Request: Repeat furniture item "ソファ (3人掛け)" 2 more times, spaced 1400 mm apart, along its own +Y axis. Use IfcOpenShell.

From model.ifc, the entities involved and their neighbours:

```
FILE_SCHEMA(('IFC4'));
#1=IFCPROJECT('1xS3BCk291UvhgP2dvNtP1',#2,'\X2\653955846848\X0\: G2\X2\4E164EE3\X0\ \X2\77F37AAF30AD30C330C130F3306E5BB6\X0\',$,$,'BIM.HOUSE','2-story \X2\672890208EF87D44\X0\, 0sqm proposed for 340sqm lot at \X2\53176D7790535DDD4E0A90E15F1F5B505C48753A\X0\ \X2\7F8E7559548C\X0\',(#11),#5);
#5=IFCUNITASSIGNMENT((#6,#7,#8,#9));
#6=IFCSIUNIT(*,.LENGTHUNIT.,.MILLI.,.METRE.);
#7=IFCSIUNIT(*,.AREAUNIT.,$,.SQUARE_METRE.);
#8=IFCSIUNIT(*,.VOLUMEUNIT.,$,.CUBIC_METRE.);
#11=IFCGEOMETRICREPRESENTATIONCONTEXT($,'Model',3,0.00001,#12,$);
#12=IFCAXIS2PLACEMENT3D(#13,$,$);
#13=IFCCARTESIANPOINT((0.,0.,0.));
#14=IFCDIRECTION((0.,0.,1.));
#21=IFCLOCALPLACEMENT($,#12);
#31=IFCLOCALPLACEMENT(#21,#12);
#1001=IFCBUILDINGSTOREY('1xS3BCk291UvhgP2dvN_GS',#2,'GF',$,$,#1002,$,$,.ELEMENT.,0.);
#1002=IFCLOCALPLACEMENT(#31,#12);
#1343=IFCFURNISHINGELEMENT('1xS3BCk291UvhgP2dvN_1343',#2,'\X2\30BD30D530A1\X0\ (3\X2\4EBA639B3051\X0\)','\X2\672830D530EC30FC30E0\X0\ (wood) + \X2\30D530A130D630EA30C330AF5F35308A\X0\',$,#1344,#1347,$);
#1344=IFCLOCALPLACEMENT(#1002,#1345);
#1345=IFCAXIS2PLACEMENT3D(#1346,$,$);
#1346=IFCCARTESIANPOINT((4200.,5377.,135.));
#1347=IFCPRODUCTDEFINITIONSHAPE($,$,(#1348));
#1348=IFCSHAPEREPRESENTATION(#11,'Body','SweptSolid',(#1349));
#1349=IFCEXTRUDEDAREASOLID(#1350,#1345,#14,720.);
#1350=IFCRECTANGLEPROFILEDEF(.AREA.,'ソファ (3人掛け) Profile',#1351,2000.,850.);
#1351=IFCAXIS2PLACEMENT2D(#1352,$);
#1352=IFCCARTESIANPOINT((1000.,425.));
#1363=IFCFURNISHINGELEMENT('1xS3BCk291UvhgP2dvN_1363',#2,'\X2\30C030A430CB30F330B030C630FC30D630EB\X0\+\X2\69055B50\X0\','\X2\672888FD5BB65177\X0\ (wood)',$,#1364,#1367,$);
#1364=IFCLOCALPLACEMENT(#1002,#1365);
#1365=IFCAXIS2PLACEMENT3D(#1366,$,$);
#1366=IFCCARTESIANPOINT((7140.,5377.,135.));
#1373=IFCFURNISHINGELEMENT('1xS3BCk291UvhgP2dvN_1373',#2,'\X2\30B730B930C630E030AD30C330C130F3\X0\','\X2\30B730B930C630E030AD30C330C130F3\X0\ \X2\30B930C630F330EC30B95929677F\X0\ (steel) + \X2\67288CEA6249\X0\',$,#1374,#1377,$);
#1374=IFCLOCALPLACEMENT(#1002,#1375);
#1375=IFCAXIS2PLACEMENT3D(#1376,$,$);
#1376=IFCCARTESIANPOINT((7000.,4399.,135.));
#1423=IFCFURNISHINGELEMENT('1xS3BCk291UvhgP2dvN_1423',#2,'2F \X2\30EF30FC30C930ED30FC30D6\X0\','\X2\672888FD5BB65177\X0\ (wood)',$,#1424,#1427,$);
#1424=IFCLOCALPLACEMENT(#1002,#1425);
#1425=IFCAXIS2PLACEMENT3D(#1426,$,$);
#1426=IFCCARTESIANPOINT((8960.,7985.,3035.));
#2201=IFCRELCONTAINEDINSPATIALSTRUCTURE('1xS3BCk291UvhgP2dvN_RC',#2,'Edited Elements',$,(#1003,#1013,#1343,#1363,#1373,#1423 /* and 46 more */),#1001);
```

```python
import ifcopenshell
import ifcopenshell.api.geometry
import ifcopenshell.api.root
import ifcopenshell.util.element
import ifcopenshell.util.placement

model = ifcopenshell.open("model.ifc")


def reuse_history(source, copy):
    """copy_class also copies each property set's owner history, people and application; keep the originals."""
    for rel in copy.IsDefinedBy:
        if rel.is_a("IfcRelDefinesByProperties") and (history := rel.RelatingPropertyDefinition.OwnerHistory):
            rel.RelatingPropertyDefinition.OwnerHistory = source.OwnerHistory
            ifcopenshell.util.element.remove_deep2(model, history)


source = model.by_guid("1xS3BCk291UvhgP2dvN_1343")
base = ifcopenshell.util.placement.get_local_placement(source.ObjectPlacement)
step = base[:3, 1] * 1400.0

for i in range(1, 3):
    copy = ifcopenshell.api.root.copy_class(model, product=source)
    copy.Representation = ifcopenshell.util.element.copy_deep(
        model, source.Representation, exclude=["IfcGeometricRepresentationContext", "IfcRepresentationMap"]
    )
    reuse_history(source, copy)
    matrix = base.copy()
    matrix[:3, 3] += i * step
    print("added at", matrix[:3, 3].round(3) + 0.0)
    ifcopenshell.api.geometry.edit_object_placement(model, product=copy, matrix=matrix, is_si=False)

model.write("model-out.ifc")
```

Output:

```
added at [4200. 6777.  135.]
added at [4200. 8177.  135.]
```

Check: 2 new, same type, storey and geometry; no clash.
